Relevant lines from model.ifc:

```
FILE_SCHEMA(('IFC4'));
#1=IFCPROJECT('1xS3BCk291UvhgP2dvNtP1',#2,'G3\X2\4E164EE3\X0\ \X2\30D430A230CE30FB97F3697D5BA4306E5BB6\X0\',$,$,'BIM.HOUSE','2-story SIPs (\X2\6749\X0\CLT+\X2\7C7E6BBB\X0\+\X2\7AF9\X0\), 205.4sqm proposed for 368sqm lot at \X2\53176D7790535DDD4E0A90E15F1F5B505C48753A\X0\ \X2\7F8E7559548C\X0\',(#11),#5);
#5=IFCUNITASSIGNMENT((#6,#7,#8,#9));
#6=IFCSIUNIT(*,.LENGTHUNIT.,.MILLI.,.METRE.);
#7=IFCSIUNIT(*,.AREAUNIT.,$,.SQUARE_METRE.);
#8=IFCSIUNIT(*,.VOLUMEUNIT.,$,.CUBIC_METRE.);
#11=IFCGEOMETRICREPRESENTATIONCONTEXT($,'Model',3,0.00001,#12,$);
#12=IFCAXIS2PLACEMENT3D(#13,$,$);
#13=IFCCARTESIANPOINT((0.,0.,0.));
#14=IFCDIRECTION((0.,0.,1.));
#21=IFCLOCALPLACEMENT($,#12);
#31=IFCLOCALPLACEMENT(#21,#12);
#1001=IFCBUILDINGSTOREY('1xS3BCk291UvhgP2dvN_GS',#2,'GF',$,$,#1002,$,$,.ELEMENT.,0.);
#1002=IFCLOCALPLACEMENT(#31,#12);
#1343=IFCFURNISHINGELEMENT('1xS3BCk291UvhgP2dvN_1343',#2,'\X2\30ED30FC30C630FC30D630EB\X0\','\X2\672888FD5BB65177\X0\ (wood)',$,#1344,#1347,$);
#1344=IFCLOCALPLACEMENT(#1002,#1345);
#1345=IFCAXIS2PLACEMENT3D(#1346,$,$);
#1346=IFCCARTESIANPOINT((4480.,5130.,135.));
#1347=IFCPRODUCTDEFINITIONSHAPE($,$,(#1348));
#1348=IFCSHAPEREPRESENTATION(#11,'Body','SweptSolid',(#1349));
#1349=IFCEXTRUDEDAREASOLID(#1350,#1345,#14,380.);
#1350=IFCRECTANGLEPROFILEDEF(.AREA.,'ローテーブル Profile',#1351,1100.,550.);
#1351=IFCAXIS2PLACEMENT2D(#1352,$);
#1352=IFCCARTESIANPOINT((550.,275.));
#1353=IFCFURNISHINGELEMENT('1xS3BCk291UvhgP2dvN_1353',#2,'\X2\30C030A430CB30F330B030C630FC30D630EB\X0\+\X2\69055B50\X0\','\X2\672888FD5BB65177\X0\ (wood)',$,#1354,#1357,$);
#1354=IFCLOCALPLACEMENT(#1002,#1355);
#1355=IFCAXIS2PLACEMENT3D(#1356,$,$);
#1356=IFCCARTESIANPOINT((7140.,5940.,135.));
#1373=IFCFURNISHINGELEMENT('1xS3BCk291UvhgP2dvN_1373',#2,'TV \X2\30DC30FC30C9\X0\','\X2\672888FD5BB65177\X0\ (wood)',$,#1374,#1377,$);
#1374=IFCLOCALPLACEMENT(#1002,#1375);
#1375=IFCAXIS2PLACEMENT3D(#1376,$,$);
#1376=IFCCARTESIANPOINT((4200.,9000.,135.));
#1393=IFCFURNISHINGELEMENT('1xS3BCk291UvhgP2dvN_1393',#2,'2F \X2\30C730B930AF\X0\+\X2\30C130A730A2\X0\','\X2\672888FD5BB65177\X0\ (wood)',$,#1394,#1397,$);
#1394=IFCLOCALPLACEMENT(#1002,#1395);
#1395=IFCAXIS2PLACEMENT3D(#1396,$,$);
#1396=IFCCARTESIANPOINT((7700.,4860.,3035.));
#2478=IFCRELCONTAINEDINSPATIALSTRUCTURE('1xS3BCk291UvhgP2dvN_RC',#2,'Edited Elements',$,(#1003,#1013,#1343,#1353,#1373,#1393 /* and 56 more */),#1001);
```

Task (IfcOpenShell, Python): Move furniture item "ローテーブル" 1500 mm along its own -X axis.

```python
import ifcopenshell
import ifcopenshell.api.geometry
import ifcopenshell.util.placement

model = ifcopenshell.open("model.ifc")

item = model.by_id(1343)
matrix = ifcopenshell.util.placement.get_local_placement(item.ObjectPlacement)
matrix[:3, 3] -= matrix[:3, 0] * 1500.0
ifcopenshell.api.geometry.edit_object_placement(model, product=item, matrix=matrix, is_si=False)

print(ifcopenshell.util.placement.get_local_placement(item.ObjectPlacement).round(3) + 0.0)

model.write("model_rev.ifc")
```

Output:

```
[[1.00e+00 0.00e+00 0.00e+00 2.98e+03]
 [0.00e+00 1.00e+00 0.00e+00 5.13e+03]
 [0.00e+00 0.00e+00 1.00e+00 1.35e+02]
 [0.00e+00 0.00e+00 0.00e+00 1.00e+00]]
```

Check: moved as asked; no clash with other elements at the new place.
